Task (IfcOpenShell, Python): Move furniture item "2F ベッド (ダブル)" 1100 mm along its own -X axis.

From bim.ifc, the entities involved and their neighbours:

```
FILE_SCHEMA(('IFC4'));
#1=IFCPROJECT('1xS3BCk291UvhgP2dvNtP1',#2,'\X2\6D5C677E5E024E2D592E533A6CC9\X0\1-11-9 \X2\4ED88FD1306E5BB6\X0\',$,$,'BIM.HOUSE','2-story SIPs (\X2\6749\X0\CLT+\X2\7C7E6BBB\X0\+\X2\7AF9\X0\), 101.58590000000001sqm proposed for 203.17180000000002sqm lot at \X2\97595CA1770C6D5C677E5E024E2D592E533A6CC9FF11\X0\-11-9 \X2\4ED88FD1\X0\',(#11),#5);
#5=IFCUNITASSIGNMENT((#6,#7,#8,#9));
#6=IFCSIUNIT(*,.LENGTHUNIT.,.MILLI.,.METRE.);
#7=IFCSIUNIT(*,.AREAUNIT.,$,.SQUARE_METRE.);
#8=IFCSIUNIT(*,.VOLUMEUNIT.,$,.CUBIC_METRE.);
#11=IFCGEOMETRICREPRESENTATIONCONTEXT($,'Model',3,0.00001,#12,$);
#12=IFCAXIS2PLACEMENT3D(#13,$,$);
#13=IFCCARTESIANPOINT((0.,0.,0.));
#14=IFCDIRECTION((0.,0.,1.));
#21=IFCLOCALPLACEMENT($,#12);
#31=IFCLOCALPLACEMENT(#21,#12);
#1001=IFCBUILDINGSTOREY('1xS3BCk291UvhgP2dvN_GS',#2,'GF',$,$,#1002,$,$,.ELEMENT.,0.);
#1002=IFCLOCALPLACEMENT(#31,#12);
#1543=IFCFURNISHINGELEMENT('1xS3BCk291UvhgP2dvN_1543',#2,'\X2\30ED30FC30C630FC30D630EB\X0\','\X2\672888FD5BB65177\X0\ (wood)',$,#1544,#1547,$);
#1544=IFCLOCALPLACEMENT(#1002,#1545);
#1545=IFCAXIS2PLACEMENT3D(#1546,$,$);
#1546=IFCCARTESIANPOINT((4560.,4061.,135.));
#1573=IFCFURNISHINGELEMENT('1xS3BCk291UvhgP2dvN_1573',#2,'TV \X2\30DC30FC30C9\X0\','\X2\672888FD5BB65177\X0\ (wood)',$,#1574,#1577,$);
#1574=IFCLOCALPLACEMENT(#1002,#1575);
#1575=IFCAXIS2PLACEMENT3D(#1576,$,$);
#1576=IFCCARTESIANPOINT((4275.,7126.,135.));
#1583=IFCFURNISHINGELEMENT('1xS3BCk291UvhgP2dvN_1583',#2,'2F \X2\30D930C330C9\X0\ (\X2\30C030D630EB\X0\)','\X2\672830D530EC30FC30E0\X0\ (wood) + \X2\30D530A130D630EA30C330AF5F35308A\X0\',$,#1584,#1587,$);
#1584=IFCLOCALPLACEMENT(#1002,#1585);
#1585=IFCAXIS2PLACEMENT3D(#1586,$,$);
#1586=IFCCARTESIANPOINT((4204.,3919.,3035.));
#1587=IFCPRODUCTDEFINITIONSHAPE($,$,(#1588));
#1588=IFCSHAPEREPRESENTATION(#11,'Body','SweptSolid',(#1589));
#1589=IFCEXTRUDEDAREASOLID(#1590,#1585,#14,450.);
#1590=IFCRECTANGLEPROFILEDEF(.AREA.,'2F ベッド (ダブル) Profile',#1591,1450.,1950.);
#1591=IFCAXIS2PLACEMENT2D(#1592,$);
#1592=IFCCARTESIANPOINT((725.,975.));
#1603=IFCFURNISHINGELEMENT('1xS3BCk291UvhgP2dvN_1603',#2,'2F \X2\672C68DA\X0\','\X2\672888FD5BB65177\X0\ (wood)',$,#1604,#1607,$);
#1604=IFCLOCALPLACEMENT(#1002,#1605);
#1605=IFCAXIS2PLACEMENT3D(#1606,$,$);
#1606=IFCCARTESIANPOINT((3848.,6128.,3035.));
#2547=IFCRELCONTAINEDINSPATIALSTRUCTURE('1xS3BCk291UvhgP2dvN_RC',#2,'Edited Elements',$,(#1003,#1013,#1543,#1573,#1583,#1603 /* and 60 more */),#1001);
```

```python
import ifcopenshell
import ifcopenshell.api.geometry
import ifcopenshell.util.placement

model = ifcopenshell.open("bim.ifc")

item = model.by_guid("1xS3BCk291UvhgP2dvN_1583")
matrix = ifcopenshell.util.placement.get_local_placement(item.ObjectPlacement)
matrix[:3, 3] -= matrix[:3, 0] * 1100.0
ifcopenshell.api.geometry.edit_object_placement(model, product=item, matrix=matrix, is_si=False)

print(ifcopenshell.util.placement.get_local_placement(item.ObjectPlacement).round(3) + 0.0)

model.write("bim_edited.ifc")
```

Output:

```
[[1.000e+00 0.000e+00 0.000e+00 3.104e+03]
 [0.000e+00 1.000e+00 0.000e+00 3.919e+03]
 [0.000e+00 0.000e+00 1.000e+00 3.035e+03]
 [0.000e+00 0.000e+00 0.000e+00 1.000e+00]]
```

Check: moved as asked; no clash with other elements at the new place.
